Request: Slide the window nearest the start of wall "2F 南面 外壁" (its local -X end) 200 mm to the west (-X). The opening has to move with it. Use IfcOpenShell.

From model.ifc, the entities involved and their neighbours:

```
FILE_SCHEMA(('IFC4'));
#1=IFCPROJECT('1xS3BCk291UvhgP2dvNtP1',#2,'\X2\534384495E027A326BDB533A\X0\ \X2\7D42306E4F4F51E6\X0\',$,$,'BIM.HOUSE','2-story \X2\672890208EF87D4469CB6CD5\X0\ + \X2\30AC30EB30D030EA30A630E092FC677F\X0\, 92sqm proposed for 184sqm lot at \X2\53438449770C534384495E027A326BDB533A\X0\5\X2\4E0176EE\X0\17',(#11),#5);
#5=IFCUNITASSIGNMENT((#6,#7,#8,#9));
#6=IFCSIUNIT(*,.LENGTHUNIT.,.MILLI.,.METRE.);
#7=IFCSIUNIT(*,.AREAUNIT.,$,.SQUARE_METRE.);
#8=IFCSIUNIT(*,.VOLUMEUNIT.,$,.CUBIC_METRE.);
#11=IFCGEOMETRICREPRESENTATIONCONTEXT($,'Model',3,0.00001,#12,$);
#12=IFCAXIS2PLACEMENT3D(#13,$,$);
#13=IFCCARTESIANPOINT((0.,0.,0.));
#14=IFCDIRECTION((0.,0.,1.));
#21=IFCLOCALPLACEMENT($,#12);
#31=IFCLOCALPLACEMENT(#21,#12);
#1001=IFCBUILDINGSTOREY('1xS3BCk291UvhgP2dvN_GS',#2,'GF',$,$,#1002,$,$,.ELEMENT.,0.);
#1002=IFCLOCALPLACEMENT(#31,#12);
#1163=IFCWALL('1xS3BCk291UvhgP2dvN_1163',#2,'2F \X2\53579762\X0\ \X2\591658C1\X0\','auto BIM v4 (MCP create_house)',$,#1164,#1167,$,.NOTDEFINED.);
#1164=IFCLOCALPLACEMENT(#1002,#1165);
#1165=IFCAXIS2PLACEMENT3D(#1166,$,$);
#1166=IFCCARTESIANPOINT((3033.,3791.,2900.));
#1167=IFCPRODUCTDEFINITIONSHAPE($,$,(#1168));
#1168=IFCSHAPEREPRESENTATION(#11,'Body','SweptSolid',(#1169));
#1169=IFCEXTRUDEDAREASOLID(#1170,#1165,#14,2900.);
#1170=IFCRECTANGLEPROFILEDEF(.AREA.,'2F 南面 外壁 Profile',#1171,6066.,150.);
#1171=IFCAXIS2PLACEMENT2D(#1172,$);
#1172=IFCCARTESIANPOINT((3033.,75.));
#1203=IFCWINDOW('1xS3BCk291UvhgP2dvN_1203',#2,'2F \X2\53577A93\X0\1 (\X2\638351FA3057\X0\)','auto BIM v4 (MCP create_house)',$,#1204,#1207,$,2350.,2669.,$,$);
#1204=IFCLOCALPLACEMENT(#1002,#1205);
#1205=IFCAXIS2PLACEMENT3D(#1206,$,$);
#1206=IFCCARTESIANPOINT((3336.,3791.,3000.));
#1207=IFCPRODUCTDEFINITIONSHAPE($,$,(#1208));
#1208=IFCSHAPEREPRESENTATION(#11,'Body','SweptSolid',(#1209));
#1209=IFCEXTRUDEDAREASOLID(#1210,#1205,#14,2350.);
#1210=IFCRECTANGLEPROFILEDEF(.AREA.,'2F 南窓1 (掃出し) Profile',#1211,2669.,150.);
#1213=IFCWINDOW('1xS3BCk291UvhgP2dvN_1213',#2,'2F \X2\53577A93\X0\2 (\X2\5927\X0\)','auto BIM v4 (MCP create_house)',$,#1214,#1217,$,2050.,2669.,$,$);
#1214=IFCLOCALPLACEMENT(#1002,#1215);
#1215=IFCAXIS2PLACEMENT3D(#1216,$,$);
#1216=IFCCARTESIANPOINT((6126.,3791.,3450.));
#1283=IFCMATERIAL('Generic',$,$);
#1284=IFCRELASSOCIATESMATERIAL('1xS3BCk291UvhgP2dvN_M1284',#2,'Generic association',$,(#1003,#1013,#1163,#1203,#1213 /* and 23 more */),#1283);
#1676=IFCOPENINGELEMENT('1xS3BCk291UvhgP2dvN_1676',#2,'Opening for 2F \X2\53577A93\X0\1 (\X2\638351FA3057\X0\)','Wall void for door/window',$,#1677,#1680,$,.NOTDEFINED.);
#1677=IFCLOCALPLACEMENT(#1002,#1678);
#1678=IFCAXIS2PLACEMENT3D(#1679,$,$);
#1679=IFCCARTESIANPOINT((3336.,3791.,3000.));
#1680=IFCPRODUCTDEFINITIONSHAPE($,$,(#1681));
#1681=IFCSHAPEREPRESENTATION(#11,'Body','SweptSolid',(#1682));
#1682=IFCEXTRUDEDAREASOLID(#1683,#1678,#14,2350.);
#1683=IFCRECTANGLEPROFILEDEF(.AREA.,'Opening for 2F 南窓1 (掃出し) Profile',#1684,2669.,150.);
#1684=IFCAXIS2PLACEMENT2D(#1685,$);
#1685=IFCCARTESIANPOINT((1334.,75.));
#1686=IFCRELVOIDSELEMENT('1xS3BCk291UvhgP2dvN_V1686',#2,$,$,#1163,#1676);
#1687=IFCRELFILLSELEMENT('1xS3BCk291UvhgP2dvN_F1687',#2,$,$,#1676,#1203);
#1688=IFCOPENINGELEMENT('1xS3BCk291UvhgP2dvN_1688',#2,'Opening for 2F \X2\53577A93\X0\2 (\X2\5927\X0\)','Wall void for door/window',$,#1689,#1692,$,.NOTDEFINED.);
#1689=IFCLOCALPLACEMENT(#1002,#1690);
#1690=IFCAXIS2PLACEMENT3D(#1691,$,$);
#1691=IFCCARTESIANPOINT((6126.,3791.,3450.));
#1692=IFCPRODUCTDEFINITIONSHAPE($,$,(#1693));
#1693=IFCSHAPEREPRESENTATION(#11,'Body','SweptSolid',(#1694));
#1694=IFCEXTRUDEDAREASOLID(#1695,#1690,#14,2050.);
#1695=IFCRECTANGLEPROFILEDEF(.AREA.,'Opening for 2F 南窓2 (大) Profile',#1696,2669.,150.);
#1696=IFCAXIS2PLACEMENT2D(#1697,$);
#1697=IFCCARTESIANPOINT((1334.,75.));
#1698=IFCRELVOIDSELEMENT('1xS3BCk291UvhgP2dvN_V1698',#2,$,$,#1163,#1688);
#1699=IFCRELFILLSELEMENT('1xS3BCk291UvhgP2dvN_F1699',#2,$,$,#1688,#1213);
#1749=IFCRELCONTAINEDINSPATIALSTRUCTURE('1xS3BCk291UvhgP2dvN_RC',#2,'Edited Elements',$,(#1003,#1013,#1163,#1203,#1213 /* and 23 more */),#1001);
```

```python
import ifcopenshell
import ifcopenshell.api.geometry
import ifcopenshell.util.placement

model = ifcopenshell.open("model.ifc")

window = model.by_guid("1xS3BCk291UvhgP2dvN_1203")
opening = window.FillsVoids[0].RelatingOpeningElement
wall = opening.VoidsElements[0].RelatingBuildingElement

wall_matrix = ifcopenshell.util.placement.get_local_placement(wall.ObjectPlacement)
shift = wall_matrix[:3, 0] * -200.0
before = ifcopenshell.util.placement.get_local_placement(window.ObjectPlacement)[:3, 3].copy()

# The window is not placed relative to its opening, so move both.
for product in (opening, window):
    matrix = ifcopenshell.util.placement.get_local_placement(product.ObjectPlacement)
    matrix[:3, 3] += shift
    ifcopenshell.api.geometry.edit_object_placement(model, product=product, matrix=matrix, is_si=False)

after = ifcopenshell.util.placement.get_local_placement(window.ObjectPlacement)[:3, 3]
print("window moved by", (after - before).round(3) + 0.0)

model.write("model_rev.ifc")
```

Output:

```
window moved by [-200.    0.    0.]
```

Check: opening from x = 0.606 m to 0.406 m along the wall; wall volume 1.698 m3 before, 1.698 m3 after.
